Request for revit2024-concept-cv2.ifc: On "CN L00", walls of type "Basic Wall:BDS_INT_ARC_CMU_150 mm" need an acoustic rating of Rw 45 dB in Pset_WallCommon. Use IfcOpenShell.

First a look at what the model holds.

```python
import ifcopenshell
import ifcopenshell.util.element

model = ifcopenshell.open("revit2024-concept-cv2.ifc")
print(model.schema)
storey = next(s for s in model.by_type("IfcBuildingStorey") if s.Name == "CN L00")
walls = [e for e in ifcopenshell.util.element.get_decomposition(storey) if e.is_a("IfcWall")]
seen = {}
for e in walls:
    element_type = ifcopenshell.util.element.get_type(e)
    key = (element_type.Name if element_type != e and element_type else None, ifcopenshell.util.element.get_pset(e, "Pset_WallCommon", "AcousticRating"))
    seen[key] = seen.get(key, 0) + 1
for (name, value), count in sorted(seen.items(), key=str):
    print(count, "x", name, "|", value)
```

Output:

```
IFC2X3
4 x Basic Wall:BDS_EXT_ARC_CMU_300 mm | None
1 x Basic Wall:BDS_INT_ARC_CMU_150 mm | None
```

```python
import ifcopenshell
import ifcopenshell.api.pset
import ifcopenshell.util.element

model = ifcopenshell.open("revit2024-concept-cv2.ifc")

storey = next(s for s in model.by_type("IfcBuildingStorey") if s.Name == "CN L00")
walls = [e for e in ifcopenshell.util.element.get_decomposition(storey) if e.is_a("IfcWall")]

count = 0
for e in walls:
    element_type = ifcopenshell.util.element.get_type(e)
    if element_type in (None, e) or element_type.Name != "Basic Wall:BDS_INT_ARC_CMU_150 mm":
        continue
    # add_pset returns the element's existing set when there is one.
    pset = ifcopenshell.api.pset.add_pset(model, product=e, name="Pset_WallCommon")
    ifcopenshell.api.pset.edit_pset(model, pset=pset, properties={"AcousticRating": "Rw 45 dB"})
    count += 1

print(count, "walls updated")

model.write("revit2024-concept-cv2_edited.ifc")
```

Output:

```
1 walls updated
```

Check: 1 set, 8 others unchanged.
